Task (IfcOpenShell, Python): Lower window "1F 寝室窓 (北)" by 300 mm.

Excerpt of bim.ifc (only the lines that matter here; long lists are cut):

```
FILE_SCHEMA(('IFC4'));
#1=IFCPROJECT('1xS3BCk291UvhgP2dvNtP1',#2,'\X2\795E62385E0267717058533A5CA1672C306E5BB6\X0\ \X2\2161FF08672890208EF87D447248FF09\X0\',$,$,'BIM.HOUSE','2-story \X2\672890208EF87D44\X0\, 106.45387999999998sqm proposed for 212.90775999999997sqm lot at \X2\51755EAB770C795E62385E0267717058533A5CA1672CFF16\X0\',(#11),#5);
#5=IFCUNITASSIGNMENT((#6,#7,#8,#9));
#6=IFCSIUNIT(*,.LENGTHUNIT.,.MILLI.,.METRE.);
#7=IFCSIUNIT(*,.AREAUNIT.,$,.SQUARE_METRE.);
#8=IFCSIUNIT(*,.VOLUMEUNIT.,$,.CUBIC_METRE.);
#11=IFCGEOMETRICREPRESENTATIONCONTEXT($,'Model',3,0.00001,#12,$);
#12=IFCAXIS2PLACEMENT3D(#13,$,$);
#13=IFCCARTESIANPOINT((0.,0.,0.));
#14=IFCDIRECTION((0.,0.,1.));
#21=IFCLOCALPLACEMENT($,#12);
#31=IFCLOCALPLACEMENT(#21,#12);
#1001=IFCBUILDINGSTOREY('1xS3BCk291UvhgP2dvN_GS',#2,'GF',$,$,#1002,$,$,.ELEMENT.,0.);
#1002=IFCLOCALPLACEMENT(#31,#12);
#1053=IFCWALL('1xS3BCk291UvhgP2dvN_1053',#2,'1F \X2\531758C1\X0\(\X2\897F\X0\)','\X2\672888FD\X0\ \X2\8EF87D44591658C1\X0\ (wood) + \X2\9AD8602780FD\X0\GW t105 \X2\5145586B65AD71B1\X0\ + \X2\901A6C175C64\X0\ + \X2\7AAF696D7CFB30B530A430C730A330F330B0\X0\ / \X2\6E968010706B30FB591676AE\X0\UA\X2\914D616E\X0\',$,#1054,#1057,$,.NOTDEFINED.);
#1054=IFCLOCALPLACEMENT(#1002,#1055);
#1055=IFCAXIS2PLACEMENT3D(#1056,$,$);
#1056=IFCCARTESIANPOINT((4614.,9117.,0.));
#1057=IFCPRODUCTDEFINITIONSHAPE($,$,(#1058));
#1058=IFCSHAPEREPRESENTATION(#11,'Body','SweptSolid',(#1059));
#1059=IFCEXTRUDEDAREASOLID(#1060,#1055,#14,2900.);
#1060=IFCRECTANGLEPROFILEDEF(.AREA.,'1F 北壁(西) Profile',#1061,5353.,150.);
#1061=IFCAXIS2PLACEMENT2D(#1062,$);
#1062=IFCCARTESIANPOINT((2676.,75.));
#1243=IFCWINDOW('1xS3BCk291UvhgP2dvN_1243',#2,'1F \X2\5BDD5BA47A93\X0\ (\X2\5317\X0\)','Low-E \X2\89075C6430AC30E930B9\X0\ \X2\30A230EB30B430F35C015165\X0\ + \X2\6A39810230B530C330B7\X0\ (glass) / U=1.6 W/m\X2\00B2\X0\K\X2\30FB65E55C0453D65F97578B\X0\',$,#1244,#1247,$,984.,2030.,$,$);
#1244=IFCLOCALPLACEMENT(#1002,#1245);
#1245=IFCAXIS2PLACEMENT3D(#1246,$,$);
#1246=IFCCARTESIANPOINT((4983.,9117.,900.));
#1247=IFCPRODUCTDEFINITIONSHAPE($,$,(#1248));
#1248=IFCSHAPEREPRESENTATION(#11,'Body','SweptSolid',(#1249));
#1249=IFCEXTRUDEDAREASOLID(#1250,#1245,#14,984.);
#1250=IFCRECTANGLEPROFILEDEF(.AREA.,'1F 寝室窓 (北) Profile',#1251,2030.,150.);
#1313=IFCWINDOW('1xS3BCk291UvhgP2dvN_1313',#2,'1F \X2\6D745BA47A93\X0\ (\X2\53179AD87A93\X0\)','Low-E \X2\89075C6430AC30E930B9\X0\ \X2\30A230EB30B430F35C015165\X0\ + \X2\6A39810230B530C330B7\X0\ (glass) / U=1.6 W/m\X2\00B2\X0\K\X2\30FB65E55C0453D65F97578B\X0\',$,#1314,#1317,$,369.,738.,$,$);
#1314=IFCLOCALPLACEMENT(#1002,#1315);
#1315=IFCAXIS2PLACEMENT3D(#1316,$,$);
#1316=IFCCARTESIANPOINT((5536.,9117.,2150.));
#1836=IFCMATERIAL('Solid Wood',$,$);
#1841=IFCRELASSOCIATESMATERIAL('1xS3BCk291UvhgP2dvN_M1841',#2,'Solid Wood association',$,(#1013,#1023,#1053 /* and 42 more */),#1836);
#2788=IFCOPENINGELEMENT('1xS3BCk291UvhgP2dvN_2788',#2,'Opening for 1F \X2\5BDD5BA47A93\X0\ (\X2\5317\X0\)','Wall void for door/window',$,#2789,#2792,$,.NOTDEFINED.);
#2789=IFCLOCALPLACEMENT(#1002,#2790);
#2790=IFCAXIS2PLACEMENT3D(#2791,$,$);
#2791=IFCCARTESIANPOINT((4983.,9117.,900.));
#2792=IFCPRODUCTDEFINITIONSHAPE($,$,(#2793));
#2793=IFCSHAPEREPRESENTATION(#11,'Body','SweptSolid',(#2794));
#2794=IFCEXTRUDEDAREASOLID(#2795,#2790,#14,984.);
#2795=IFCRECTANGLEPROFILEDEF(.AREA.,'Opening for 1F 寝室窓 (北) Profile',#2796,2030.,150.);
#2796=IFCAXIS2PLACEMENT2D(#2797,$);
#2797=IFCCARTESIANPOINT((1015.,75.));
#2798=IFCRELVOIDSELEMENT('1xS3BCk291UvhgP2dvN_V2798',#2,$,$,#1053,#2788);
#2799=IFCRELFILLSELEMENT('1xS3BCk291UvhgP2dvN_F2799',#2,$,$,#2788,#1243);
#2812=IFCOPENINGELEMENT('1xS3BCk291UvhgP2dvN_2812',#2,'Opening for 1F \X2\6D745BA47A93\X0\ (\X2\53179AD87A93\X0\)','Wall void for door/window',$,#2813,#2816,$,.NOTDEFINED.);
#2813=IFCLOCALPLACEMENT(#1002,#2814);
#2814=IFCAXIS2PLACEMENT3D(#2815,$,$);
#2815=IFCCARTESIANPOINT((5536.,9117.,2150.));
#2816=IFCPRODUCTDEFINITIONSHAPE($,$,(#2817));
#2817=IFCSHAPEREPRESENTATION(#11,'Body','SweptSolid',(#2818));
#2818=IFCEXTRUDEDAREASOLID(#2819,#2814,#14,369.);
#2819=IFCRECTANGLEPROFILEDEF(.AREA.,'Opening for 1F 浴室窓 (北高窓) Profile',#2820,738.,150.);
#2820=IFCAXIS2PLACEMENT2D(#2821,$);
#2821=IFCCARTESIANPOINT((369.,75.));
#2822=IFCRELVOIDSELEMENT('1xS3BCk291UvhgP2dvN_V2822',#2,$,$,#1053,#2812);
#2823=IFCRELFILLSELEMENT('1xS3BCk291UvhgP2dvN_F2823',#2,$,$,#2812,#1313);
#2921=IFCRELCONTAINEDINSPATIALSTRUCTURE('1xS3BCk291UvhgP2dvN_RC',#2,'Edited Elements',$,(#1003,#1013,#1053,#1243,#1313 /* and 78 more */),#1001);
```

```python
import numpy as np
import ifcopenshell
import ifcopenshell.api.geometry
import ifcopenshell.util.placement
import ifcopenshell.util.unit

model = ifcopenshell.open("bim.ifc")
unit_scale = ifcopenshell.util.unit.calculate_unit_scale(model)

window = model.by_guid("1xS3BCk291UvhgP2dvN_1243")
opening = window.FillsVoids[0].RelatingOpeningElement
dz = -0.3 / unit_scale

shift = np.array([0.0, 0.0, dz])
# The window is not placed relative to its opening, so move both.
for product in (opening, window):
    matrix = ifcopenshell.util.placement.get_local_placement(product.ObjectPlacement)
    matrix[:3, 3] += shift
    ifcopenshell.api.geometry.edit_object_placement(model, product=product, matrix=matrix, is_si=False)

print(f"moved by {dz * unit_scale:+.3f} m")

model.write("bim_rev.ifc")
```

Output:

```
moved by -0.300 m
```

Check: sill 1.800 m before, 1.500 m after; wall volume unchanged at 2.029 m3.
